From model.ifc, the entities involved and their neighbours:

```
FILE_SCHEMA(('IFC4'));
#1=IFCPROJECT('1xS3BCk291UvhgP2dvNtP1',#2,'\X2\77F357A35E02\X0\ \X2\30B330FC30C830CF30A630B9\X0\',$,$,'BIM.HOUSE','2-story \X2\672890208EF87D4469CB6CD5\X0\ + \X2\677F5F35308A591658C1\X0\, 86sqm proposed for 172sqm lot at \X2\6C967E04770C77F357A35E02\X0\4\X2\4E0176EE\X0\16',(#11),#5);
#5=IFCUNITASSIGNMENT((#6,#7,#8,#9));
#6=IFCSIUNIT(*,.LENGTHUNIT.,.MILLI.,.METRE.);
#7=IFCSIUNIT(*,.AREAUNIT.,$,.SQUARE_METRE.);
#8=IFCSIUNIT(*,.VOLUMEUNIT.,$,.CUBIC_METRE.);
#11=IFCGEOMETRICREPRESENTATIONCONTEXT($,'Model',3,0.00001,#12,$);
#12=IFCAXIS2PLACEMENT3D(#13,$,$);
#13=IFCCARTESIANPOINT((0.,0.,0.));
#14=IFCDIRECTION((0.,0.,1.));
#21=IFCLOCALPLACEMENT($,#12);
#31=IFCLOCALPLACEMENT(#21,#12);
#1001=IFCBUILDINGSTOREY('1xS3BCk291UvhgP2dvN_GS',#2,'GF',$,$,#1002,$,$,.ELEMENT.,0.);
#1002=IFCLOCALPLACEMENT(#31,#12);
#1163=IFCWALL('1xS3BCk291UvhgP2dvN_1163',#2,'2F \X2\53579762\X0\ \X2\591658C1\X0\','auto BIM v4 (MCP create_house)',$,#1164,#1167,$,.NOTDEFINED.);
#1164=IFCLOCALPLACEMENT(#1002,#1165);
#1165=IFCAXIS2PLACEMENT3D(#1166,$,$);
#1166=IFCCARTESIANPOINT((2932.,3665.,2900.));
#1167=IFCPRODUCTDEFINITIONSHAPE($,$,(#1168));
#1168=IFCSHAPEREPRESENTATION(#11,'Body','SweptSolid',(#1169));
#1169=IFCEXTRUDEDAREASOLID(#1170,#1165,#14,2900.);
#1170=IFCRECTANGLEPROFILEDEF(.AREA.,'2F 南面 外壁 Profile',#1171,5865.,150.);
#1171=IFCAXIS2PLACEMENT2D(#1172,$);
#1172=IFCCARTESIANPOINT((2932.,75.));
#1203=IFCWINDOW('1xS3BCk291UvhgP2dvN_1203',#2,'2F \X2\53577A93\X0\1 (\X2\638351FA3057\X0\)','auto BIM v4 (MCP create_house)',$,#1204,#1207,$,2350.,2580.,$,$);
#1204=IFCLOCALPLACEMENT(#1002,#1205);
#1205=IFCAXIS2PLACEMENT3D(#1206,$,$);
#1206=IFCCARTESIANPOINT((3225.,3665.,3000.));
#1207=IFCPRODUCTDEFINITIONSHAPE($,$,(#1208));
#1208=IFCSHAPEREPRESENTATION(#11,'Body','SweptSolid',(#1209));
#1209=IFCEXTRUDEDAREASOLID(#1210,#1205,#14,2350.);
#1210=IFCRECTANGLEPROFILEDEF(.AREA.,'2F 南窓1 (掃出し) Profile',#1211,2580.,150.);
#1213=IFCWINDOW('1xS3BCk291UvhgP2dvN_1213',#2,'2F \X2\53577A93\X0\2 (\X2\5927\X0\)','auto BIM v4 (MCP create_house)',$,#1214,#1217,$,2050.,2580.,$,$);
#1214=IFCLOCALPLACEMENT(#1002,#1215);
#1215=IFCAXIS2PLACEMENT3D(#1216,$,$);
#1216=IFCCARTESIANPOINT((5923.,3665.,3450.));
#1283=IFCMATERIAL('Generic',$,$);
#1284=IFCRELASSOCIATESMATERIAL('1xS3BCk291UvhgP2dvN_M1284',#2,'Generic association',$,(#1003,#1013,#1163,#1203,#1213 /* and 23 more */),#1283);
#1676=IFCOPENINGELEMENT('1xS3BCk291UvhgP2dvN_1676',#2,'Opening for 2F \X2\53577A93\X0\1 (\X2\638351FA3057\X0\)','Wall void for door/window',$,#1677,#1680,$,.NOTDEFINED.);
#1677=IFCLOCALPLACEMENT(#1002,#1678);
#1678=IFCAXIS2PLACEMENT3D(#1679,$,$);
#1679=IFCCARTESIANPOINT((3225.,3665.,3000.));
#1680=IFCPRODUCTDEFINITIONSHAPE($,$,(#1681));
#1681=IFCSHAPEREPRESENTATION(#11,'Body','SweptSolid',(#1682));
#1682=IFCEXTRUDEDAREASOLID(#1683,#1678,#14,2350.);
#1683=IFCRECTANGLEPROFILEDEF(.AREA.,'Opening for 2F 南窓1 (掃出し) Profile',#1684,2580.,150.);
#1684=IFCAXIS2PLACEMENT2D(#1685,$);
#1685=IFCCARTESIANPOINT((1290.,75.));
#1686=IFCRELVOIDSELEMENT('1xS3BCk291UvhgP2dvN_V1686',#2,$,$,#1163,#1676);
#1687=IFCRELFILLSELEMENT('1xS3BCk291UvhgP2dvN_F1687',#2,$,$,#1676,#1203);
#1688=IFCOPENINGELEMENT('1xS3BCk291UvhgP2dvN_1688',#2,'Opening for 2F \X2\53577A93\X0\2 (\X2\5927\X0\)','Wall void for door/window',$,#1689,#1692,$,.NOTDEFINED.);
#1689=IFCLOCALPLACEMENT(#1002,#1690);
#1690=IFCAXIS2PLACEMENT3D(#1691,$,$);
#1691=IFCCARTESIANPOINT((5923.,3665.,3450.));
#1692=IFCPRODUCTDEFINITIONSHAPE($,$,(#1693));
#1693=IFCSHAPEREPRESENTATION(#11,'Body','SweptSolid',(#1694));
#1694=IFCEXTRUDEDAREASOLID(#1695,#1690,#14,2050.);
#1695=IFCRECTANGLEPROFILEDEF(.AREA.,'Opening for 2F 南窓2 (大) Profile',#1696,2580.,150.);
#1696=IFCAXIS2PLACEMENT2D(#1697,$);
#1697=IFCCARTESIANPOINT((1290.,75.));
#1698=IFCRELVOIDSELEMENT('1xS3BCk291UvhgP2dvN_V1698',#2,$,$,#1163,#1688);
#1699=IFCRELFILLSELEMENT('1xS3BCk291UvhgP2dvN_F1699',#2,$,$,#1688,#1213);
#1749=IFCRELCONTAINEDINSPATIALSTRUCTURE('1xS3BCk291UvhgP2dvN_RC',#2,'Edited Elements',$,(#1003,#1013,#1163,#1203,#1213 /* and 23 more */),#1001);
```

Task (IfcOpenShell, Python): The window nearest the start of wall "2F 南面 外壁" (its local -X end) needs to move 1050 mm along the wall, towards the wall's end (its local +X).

```python
import ifcopenshell
import ifcopenshell.api.geometry
import ifcopenshell.util.placement
import ifcopenshell.util.unit

model = ifcopenshell.open("model.ifc")
unit_scale = ifcopenshell.util.unit.calculate_unit_scale(model)

window = model.by_id(1203)
opening = window.FillsVoids[0].RelatingOpeningElement
wall = opening.VoidsElements[0].RelatingBuildingElement

wall_matrix = ifcopenshell.util.placement.get_local_placement(wall.ObjectPlacement)
shift = wall_matrix[:3, 0] * 1.05 / unit_scale
before = ifcopenshell.util.placement.get_local_placement(window.ObjectPlacement)[:3, 3].copy()

# The window is not placed relative to its opening, so move both.
for product in (opening, window):
    matrix = ifcopenshell.util.placement.get_local_placement(product.ObjectPlacement)
    matrix[:3, 3] += shift
    ifcopenshell.api.geometry.edit_object_placement(model, product=product, matrix=matrix, is_si=False)

after = ifcopenshell.util.placement.get_local_placement(window.ObjectPlacement)[:3, 3]
print("window moved by", (after - before).round(3) + 0.0)

model.write("model-out.ifc")
```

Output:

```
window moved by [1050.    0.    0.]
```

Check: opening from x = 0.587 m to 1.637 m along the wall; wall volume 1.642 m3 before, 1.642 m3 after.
